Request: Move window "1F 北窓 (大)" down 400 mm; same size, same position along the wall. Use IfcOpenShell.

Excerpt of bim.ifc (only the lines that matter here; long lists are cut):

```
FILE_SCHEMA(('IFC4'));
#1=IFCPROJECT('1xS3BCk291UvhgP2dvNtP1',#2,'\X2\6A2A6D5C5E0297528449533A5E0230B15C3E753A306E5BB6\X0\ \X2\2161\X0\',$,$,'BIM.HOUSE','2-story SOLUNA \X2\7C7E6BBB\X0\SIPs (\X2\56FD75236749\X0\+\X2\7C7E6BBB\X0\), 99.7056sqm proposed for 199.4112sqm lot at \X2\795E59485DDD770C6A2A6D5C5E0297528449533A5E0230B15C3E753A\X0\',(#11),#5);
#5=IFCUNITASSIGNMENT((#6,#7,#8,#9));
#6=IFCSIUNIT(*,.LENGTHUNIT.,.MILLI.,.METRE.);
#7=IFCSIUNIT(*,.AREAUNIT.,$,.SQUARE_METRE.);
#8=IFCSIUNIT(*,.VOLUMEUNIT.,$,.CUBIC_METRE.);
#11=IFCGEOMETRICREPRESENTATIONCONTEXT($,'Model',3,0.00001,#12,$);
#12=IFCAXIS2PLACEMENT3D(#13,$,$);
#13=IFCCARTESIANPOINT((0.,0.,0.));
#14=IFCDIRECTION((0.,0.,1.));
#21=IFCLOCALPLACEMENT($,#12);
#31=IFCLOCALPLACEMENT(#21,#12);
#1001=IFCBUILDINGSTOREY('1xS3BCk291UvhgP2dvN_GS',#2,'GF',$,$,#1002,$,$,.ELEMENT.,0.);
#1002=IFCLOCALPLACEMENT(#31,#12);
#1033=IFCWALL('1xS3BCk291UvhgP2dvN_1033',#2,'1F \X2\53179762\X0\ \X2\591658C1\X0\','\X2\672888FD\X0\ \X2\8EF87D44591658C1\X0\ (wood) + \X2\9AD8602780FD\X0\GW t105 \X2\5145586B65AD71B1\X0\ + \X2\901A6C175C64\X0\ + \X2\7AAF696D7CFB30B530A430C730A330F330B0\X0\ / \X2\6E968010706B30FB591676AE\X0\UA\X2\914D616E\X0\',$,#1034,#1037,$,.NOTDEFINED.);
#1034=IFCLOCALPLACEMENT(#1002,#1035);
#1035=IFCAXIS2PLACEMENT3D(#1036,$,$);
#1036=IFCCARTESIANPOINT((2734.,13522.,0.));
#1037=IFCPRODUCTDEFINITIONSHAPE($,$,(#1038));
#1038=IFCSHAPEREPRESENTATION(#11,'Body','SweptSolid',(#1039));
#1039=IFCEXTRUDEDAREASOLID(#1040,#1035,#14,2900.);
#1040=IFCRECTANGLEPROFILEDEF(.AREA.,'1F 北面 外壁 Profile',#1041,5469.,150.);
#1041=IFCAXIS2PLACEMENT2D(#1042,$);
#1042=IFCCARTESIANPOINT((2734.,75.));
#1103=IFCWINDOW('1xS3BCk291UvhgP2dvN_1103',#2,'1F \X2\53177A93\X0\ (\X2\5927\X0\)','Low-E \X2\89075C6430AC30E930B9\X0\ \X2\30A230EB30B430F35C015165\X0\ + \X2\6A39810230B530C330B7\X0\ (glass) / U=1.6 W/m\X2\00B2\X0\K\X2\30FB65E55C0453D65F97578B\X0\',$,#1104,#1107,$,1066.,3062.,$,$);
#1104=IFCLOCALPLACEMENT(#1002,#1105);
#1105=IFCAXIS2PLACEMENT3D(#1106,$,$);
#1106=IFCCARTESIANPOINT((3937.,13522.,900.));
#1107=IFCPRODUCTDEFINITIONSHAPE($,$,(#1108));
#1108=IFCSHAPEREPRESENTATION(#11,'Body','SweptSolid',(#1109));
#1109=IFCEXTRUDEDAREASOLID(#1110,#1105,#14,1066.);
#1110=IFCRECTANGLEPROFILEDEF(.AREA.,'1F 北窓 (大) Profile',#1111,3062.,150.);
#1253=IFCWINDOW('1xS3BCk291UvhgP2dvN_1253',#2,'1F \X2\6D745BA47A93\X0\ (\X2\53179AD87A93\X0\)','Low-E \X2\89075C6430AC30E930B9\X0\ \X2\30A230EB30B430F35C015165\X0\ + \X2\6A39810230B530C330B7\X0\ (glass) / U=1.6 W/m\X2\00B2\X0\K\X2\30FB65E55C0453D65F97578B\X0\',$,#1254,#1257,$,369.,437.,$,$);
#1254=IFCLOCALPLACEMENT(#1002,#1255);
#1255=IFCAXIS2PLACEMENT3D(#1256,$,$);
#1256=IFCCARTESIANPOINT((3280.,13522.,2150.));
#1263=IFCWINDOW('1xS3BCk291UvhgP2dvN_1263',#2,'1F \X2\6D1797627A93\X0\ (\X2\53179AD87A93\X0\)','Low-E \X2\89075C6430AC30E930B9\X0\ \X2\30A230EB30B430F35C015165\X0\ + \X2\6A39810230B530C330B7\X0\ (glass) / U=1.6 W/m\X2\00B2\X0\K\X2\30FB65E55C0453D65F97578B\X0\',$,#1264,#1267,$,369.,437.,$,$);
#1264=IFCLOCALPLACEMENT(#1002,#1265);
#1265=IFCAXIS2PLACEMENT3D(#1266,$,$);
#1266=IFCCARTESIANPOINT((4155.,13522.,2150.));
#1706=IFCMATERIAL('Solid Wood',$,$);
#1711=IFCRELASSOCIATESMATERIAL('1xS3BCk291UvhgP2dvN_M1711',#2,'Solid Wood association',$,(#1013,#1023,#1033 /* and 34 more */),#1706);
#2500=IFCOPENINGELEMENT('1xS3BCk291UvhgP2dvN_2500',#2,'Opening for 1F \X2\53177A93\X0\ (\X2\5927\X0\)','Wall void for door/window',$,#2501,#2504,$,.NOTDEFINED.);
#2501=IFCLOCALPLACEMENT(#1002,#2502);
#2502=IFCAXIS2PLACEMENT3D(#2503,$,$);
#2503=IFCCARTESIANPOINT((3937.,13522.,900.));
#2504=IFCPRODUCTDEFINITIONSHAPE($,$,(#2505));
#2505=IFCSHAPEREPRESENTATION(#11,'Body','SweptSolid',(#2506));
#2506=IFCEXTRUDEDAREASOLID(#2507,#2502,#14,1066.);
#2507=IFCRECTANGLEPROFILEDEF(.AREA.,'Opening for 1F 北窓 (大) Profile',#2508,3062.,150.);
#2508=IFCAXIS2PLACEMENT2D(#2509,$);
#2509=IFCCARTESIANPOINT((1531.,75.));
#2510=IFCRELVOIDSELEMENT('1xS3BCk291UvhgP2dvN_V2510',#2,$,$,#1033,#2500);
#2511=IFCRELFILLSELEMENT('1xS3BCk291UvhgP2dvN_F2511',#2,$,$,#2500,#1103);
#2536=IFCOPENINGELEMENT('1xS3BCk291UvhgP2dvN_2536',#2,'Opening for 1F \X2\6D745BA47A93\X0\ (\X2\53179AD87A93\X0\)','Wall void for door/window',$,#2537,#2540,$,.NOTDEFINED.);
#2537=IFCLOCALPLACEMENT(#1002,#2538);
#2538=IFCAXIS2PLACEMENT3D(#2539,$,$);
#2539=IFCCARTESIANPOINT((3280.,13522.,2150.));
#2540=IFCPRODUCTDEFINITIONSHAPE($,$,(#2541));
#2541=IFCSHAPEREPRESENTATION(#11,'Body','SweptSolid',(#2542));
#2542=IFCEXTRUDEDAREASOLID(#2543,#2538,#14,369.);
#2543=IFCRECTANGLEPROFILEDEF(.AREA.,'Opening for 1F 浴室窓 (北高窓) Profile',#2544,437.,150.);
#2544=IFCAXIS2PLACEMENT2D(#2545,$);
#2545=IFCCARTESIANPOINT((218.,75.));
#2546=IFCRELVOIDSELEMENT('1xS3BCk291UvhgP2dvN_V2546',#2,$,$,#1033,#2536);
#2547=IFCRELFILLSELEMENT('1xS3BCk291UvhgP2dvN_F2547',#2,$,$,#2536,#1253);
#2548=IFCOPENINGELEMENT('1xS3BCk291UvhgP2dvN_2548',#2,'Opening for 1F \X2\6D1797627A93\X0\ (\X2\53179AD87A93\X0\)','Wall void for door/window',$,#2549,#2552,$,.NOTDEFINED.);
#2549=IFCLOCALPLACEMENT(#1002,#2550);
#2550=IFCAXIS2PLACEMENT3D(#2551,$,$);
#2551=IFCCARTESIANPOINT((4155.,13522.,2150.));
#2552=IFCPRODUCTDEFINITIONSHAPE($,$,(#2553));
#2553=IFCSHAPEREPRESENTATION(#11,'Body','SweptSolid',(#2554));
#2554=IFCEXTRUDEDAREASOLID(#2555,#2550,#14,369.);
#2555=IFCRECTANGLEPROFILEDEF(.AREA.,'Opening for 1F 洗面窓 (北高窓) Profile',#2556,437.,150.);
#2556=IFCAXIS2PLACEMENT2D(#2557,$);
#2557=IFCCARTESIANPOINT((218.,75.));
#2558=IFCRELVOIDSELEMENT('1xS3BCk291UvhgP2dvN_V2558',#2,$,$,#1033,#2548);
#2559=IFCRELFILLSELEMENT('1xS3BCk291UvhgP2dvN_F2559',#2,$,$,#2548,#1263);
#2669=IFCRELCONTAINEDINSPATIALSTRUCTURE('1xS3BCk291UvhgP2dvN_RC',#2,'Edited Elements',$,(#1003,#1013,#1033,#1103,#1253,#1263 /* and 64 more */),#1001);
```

```python
import numpy as np
import ifcopenshell
import ifcopenshell.api.geometry
import ifcopenshell.util.placement
import ifcopenshell.util.unit

model = ifcopenshell.open("bim.ifc")
unit_scale = ifcopenshell.util.unit.calculate_unit_scale(model)

window = model.by_guid("1xS3BCk291UvhgP2dvN_1103")
opening = window.FillsVoids[0].RelatingOpeningElement
dz = -400.0

shift = np.array([0.0, 0.0, dz])
# The window is not placed relative to its opening, so move both.
for product in (opening, window):
    matrix = ifcopenshell.util.placement.get_local_placement(product.ObjectPlacement)
    matrix[:3, 3] += shift
    ifcopenshell.api.geometry.edit_object_placement(model, product=product, matrix=matrix, is_si=False)

print(f"moved by {dz * unit_scale:+.3f} m")

model.write("bim_edited.ifc")
```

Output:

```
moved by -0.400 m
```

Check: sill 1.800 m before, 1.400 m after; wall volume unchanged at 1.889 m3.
